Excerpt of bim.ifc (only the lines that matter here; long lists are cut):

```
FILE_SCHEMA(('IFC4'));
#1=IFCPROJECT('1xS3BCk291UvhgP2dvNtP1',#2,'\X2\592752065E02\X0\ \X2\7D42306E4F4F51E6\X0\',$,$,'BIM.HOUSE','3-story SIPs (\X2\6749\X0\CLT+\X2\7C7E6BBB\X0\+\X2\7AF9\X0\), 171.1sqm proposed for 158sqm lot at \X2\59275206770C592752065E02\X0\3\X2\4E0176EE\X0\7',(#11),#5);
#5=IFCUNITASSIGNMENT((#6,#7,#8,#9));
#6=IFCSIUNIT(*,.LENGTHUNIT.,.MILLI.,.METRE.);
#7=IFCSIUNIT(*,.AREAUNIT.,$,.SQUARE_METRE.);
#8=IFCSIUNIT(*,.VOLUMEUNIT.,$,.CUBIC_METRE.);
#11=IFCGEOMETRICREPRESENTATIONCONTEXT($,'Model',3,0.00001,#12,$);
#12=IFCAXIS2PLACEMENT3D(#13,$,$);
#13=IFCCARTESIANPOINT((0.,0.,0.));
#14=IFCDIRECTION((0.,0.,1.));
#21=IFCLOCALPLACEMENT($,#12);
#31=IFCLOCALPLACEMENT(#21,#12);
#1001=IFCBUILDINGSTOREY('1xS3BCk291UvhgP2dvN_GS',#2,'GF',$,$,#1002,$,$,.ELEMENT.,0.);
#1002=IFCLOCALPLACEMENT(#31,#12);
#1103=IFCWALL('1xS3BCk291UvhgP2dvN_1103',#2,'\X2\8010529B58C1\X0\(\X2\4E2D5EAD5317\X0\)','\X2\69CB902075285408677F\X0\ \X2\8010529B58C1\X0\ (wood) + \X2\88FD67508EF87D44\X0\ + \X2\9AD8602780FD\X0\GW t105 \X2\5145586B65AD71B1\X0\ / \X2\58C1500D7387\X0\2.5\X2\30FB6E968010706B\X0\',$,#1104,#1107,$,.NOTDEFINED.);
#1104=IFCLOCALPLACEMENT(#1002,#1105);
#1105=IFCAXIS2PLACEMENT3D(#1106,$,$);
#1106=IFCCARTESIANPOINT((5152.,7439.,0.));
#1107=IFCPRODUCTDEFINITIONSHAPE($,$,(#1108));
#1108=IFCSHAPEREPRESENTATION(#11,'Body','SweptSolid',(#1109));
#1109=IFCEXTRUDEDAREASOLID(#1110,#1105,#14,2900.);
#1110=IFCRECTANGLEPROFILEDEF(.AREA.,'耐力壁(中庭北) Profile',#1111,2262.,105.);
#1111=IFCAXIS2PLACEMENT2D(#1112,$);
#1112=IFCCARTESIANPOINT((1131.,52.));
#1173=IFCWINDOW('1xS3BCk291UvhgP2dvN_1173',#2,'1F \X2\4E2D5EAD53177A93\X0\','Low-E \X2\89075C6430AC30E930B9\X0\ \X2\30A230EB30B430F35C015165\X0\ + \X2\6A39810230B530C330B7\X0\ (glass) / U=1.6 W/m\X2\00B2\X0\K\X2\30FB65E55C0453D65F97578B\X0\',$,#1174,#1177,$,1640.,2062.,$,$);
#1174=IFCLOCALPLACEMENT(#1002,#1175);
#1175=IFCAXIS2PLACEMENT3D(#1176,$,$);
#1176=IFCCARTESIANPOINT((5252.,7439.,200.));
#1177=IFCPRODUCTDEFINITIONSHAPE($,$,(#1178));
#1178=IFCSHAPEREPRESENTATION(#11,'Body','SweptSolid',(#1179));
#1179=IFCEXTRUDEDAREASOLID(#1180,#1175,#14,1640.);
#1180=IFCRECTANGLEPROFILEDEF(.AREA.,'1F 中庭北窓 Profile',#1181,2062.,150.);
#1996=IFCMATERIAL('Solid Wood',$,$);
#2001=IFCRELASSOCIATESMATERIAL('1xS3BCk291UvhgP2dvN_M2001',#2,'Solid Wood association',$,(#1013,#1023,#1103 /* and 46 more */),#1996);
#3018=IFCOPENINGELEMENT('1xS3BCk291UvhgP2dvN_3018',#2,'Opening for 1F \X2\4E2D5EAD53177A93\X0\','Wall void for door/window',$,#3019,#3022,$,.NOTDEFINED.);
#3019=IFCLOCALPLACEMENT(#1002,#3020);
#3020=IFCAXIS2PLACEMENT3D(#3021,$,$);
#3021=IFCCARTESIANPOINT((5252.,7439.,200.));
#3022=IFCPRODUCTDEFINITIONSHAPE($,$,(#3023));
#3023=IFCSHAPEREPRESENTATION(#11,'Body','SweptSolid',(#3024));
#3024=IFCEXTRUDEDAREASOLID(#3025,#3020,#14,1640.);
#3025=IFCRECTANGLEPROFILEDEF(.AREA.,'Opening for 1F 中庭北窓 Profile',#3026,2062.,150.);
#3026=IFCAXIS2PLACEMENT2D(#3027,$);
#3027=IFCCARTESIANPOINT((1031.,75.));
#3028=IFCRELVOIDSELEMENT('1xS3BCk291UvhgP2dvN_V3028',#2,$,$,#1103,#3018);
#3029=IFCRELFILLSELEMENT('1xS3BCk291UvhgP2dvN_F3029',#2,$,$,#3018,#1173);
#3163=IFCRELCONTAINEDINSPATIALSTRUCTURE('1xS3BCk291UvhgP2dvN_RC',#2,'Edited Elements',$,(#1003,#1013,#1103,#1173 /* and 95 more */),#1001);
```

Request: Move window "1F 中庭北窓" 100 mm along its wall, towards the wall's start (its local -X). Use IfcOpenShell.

```python
import ifcopenshell
import ifcopenshell.api.geometry
import ifcopenshell.util.placement
import ifcopenshell.util.unit

model = ifcopenshell.open("bim.ifc")
unit_scale = ifcopenshell.util.unit.calculate_unit_scale(model)

window = model.by_guid("1xS3BCk291UvhgP2dvN_1173")
opening = window.FillsVoids[0].RelatingOpeningElement
wall = opening.VoidsElements[0].RelatingBuildingElement

wall_matrix = ifcopenshell.util.placement.get_local_placement(wall.ObjectPlacement)
shift = wall_matrix[:3, 0] * -0.1 / unit_scale
before = ifcopenshell.util.placement.get_local_placement(window.ObjectPlacement)[:3, 3].copy()

# The window is not placed relative to its opening, so move both.
for product in (opening, window):
    matrix = ifcopenshell.util.placement.get_local_placement(product.ObjectPlacement)
    matrix[:3, 3] += shift
    ifcopenshell.api.geometry.edit_object_placement(model, product=product, matrix=matrix, is_si=False)

after = ifcopenshell.util.placement.get_local_placement(window.ObjectPlacement)[:3, 3]
print("window moved by", (after - before).round(3) + 0.0)

model.write("bim_updated.ifc")
```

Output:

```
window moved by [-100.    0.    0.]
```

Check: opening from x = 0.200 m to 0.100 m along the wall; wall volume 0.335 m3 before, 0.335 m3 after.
